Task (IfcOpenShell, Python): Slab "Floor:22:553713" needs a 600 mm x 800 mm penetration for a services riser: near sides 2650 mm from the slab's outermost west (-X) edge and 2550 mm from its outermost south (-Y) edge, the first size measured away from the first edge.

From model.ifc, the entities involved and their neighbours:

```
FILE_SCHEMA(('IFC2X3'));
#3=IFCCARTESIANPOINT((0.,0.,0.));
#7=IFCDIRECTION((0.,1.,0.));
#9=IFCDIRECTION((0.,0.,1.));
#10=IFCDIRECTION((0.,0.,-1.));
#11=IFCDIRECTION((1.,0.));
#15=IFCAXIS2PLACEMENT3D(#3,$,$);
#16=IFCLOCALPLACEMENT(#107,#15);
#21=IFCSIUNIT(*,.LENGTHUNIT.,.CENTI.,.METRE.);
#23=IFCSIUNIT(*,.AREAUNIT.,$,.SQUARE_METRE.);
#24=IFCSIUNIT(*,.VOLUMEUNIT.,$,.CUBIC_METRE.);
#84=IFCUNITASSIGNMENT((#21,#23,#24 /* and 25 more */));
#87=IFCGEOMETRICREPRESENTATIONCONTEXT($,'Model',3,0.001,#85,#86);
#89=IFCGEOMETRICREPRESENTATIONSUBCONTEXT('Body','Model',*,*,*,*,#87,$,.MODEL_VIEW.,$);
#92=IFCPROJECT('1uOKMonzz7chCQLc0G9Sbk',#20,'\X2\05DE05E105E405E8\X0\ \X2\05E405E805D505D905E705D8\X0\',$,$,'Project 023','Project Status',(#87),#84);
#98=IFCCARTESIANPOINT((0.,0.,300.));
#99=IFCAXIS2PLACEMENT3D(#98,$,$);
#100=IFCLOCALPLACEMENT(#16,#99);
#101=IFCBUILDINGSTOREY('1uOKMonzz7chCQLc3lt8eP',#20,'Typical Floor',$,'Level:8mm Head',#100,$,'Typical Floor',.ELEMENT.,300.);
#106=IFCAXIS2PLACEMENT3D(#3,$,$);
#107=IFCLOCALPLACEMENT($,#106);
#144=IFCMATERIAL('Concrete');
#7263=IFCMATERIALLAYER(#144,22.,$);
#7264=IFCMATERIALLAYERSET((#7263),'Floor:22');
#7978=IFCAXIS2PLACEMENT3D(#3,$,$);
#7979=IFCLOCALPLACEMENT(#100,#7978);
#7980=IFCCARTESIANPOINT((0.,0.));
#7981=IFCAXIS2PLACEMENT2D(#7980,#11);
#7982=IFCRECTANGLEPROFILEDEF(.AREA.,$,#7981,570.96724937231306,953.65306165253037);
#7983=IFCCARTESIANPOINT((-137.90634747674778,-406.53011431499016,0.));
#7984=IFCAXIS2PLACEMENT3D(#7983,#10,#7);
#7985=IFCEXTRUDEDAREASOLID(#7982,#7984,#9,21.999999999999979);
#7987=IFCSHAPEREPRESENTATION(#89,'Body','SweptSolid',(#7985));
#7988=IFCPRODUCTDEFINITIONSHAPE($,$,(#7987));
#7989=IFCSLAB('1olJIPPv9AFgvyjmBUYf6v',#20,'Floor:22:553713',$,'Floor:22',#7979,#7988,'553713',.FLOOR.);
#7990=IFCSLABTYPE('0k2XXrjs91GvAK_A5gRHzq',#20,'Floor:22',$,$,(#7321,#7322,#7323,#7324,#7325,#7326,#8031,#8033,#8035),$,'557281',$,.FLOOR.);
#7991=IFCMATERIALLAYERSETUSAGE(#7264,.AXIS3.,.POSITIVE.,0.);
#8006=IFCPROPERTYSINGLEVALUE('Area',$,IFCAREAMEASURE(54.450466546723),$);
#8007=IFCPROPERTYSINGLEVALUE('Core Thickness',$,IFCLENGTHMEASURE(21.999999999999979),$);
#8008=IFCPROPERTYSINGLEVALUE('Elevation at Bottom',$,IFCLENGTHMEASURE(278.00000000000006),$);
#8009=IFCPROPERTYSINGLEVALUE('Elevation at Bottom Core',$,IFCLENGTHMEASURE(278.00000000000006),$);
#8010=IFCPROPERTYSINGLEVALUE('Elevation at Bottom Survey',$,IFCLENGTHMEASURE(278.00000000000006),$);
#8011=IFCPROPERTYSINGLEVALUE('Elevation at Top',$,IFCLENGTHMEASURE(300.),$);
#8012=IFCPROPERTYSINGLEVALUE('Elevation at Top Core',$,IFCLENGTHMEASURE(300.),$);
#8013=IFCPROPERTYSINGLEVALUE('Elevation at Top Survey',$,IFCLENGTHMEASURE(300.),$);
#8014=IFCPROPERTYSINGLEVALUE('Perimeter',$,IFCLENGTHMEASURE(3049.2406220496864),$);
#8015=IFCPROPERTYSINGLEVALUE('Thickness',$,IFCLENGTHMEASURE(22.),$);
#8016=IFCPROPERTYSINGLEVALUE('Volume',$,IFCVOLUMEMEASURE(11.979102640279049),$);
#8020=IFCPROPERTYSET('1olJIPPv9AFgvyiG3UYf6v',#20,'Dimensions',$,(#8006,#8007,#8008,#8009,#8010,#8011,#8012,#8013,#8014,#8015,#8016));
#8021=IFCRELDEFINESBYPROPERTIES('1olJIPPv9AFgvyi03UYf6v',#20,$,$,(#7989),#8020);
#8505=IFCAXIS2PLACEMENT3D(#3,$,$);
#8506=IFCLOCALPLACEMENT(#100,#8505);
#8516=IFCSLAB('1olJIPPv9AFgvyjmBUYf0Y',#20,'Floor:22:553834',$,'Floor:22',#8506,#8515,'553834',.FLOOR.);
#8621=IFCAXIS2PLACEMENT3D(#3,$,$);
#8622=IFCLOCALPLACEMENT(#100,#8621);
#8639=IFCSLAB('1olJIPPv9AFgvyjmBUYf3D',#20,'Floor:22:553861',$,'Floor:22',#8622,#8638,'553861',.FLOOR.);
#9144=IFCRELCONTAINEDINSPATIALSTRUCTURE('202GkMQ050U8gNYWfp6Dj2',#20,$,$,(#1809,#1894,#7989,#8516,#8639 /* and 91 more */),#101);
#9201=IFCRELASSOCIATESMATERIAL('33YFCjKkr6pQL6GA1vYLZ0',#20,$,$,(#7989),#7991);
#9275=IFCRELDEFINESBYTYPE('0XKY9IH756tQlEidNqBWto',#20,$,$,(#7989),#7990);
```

```python
import numpy as np
import ifcopenshell
import ifcopenshell.api.feature
import ifcopenshell.api.geometry
import ifcopenshell.api.pset
import ifcopenshell.api.root
import ifcopenshell.geom
import ifcopenshell.util.element
import ifcopenshell.util.placement
import ifcopenshell.util.representation
import ifcopenshell.util.shape
import ifcopenshell.util.unit

model = ifcopenshell.open("model.ifc")
unit_scale = ifcopenshell.util.unit.calculate_unit_scale(model)
area_scale = ifcopenshell.util.unit.calculate_unit_scale(model, "AREAUNIT")
volume_scale = ifcopenshell.util.unit.calculate_unit_scale(model, "VOLUMEUNIT")
settings = ifcopenshell.geom.settings()


def volume(element):
    """Net volume in cubic metres, openings subtracted."""
    shape = ifcopenshell.geom.create_shape(settings, element)
    return ifcopenshell.util.shape.get_volume(shape.geometry)


slab = model.by_guid("1olJIPPv9AFgvyjmBUYf6v")
before = volume(slab)

# Extent in the slab's own axes, in metres. The edges named are its -X and -Y sides.
slab_shape = ifcopenshell.geom.create_shape(settings, slab)
vertices = ifcopenshell.util.shape.get_vertices(slab_shape.geometry)
x_min, y_min, bottom = vertices.min(axis=0)
top = vertices[:, 2].max()

opening = ifcopenshell.api.root.create_entity(model, ifc_class="IfcOpeningElement", name="Services riser opening")
context = ifcopenshell.util.representation.get_context(model, "Model", "Body", "MODEL_VIEW")
width, depth = 0.6, 0.8
outline = [(0.0, 0.0), (width, 0.0), (width, depth), (0.0, depth), (0.0, 0.0)]
# Overshoot both faces by 50 mm so the cut is clean.
shape = ifcopenshell.api.geometry.add_slab_representation(
    model, context=context, depth=top - bottom + 0.1, polyline=outline
)
ifcopenshell.api.geometry.assign_representation(model, product=opening, representation=shape)

matrix = ifcopenshell.util.placement.get_local_placement(slab.ObjectPlacement)
matrix[:, 3] = matrix @ np.append(np.array([x_min + 2.65, y_min + 2.55, bottom - 0.05]) / unit_scale, 1.0)
ifcopenshell.api.geometry.edit_object_placement(model, product=opening, matrix=matrix, is_si=False)
ifcopenshell.api.feature.add_feature(model, feature=opening, element=slab)

after = volume(slab)

# Update the slab's stored quantities.
pset = model.by_id(ifcopenshell.util.element.get_pset(slab, "Dimensions", should_inherit=False)["id"])
ifcopenshell.api.pset.edit_pset(model, pset=pset, properties={
    "Area": model.create_entity("IfcAreaMeasure", after / (top - bottom) / area_scale),
    "Volume": model.create_entity("IfcVolumeMeasure", after / volume_scale),
})

print(f"slab volume {before:.3f} -> {after:.3f} m3")

model.write("model-out.ifc")
```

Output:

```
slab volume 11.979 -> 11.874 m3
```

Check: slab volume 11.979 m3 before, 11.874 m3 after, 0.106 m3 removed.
